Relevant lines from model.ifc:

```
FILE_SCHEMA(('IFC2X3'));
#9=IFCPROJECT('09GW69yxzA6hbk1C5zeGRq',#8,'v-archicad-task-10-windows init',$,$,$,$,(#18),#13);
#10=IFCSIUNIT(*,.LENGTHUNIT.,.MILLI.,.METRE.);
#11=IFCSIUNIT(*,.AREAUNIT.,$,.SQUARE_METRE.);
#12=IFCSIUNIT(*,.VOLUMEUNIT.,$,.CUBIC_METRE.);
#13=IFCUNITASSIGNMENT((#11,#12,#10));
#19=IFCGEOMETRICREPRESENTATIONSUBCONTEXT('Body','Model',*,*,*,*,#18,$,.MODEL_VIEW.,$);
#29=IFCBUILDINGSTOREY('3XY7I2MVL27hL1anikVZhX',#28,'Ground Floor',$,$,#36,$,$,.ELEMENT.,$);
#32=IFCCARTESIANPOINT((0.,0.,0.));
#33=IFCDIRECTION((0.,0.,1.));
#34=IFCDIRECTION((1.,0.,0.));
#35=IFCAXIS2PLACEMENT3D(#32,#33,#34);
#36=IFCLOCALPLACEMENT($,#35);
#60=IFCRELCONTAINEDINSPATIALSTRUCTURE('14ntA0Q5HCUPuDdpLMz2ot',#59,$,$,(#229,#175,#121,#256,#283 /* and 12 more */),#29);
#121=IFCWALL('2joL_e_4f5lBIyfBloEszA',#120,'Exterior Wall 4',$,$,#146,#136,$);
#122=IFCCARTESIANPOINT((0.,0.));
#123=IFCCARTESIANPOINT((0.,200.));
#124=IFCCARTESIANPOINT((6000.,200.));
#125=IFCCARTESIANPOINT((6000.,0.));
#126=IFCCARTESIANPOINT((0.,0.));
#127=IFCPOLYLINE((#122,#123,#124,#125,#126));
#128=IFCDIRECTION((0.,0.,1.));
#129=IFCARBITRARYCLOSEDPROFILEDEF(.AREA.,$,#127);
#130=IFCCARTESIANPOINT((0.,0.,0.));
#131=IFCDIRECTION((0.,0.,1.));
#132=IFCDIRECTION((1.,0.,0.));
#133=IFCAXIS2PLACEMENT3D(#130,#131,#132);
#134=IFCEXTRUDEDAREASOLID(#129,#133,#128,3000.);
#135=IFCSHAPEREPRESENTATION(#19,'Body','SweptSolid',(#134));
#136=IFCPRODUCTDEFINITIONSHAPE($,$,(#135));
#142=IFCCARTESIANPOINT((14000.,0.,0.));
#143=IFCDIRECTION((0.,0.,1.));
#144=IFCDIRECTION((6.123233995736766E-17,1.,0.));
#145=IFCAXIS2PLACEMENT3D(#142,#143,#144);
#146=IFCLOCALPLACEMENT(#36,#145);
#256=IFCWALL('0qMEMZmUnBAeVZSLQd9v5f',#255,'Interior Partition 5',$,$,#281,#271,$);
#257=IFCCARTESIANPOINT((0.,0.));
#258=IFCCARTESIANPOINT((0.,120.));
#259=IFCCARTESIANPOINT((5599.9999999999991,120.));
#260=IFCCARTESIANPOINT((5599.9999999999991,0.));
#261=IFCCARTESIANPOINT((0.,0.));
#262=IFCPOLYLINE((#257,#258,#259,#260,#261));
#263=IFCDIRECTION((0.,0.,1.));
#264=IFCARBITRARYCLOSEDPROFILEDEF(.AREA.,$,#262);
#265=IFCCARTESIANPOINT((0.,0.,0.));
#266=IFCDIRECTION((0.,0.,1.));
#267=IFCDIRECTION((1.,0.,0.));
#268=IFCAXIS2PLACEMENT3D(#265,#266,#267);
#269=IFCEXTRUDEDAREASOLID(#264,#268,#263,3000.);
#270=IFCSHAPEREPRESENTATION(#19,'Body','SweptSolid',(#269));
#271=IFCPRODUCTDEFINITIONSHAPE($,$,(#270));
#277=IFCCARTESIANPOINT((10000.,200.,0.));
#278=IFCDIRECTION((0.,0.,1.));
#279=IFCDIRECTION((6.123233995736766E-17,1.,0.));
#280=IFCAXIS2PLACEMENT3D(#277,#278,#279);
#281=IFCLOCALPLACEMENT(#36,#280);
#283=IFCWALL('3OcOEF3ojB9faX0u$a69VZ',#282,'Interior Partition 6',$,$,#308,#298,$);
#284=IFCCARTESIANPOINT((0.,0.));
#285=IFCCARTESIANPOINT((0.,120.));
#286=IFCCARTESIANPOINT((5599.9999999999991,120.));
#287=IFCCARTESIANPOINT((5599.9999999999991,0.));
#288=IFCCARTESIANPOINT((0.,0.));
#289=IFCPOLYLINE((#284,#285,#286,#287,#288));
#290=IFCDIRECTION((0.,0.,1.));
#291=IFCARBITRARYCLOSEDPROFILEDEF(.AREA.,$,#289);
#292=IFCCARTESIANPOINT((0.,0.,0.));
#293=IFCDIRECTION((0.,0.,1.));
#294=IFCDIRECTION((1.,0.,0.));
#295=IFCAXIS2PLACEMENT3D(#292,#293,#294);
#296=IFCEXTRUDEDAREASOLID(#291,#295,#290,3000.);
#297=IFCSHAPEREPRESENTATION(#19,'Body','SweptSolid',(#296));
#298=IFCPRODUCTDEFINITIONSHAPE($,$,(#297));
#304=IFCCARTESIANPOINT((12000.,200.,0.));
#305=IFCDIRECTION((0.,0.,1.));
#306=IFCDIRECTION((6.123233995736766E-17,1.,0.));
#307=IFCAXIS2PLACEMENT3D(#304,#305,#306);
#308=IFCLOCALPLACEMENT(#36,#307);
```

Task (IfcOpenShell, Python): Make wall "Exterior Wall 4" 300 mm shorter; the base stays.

```python
import ifcopenshell
import ifcopenshell.geom
import ifcopenshell.util.representation
import ifcopenshell.util.shape
import ifcopenshell.util.unit

model = ifcopenshell.open("model.ifc")
unit_scale = ifcopenshell.util.unit.calculate_unit_scale(model)
settings = ifcopenshell.geom.settings()


def volume(element):
    """Net volume in cubic metres, openings subtracted."""
    shape = ifcopenshell.geom.create_shape(settings, element)
    return ifcopenshell.util.shape.get_volume(shape.geometry)


wall = model.by_id(121)
before = volume(wall)

body = ifcopenshell.util.representation.get_representation(wall, "Model", "Body")
solid = body.Items[0]
old_height = solid.Depth
solid.Depth -= 0.3 / unit_scale
after = volume(wall)

print(f"height {old_height:g} -> {solid.Depth:g}, volume {before:.3f} -> {after:.3f} m3")

model.write("model_edited.ifc")
```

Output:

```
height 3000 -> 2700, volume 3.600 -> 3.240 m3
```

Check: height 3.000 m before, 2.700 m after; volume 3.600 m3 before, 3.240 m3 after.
